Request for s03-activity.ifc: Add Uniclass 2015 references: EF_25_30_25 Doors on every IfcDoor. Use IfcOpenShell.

First a look at what the model holds.

```python
import ifcopenshell

model = ifcopenshell.open("s03-activity.ifc")
print(model.schema)
print("classifications:", [c.Name for c in model.by_type("IfcClassification")])
for ifc_class in ("IfcDoor", "IfcRoof", "IfcStair", "IfcWall", "IfcWindow"):
    print(ifc_class, len(model.by_type(ifc_class)))
```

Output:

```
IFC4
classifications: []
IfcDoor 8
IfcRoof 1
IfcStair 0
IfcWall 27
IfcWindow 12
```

```python
import ifcopenshell
import ifcopenshell.api.classification

model = ifcopenshell.open("s03-activity.ifc")

system = ifcopenshell.api.classification.add_classification(model, classification="Uniclass 2015")

codes = {
    "IfcDoor": ("EF_25_30_25", "Doors"),
}
for ifc_class, (code, name) in codes.items():
    products = model.by_type(ifc_class)
    ifcopenshell.api.classification.add_reference(
        model, products=products, classification=system, identification=code, name=name
    )
    print(code, len(products))

model.write("s03-activity_edited.ifc")
```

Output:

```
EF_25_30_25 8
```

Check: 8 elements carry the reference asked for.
